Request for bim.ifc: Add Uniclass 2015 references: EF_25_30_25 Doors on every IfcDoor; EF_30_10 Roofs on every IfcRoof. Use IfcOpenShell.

First a look at what the model holds.

```python
import ifcopenshell

model = ifcopenshell.open("bim.ifc")
print(model.schema)
print("classifications:", [c.Name for c in model.by_type("IfcClassification")])
for ifc_class in ("IfcDoor", "IfcRoof", "IfcStair", "IfcWall", "IfcWindow"):
    print(ifc_class, len(model.by_type(ifc_class)))
```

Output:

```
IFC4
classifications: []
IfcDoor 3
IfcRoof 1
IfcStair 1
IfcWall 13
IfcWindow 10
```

```python
import ifcopenshell
import ifcopenshell.api.classification

model = ifcopenshell.open("bim.ifc")

system = ifcopenshell.api.classification.add_classification(model, classification="Uniclass 2015")

codes = {
    "IfcDoor": ("EF_25_30_25", "Doors"),
    "IfcRoof": ("EF_30_10", "Roofs"),
}
for ifc_class, (code, name) in codes.items():
    products = model.by_type(ifc_class)
    ifcopenshell.api.classification.add_reference(
        model, products=products, classification=system, identification=code, name=name
    )
    print(code, len(products))

model.write("bim-out.ifc")
```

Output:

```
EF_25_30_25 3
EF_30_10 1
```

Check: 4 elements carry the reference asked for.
